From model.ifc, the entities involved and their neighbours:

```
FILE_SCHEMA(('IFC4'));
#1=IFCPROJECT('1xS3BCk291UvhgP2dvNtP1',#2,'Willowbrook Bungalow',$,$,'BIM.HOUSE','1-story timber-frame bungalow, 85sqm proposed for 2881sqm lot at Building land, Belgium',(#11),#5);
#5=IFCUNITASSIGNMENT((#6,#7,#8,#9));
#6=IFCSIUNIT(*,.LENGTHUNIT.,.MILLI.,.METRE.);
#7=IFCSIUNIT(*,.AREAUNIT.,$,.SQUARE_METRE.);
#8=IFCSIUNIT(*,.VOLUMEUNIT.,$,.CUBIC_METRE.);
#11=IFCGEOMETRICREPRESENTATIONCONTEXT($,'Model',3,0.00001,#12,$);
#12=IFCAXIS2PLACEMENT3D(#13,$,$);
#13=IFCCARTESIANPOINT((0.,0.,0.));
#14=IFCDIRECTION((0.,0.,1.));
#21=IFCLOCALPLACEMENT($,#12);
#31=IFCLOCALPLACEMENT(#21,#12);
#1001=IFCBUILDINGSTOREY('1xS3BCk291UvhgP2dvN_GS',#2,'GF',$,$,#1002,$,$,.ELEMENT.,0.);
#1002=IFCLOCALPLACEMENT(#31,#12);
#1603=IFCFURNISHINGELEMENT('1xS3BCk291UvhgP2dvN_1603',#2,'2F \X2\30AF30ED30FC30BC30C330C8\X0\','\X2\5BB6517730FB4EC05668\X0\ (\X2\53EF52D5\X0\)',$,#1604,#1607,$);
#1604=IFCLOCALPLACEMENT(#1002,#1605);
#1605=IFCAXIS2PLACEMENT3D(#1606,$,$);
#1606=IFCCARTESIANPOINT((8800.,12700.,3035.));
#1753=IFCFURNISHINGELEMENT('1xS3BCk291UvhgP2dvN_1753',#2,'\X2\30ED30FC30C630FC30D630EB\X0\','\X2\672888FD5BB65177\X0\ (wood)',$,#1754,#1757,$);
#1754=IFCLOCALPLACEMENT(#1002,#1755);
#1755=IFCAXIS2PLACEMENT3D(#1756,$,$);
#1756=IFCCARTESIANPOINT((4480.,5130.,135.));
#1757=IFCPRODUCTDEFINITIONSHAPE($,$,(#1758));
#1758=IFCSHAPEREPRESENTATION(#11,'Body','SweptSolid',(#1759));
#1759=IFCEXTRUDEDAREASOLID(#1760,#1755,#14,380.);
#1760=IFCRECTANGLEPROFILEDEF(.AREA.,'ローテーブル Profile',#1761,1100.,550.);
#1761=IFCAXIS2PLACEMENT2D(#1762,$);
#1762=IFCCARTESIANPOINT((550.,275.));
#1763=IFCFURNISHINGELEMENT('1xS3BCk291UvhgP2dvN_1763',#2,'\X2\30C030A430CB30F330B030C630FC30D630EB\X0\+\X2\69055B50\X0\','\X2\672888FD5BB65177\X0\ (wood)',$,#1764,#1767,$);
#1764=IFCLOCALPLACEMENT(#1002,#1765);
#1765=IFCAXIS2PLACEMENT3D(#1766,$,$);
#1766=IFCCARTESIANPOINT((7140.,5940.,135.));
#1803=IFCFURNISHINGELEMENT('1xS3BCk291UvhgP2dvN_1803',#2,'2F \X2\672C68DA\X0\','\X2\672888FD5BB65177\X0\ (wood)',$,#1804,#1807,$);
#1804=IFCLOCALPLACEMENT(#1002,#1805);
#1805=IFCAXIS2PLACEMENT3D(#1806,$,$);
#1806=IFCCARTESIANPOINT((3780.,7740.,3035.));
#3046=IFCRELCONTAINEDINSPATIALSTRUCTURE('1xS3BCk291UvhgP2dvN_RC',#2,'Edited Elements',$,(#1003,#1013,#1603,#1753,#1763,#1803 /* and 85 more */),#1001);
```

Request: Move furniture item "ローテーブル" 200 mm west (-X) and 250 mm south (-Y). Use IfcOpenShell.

```python
import ifcopenshell
import ifcopenshell.api.geometry
import ifcopenshell.util.placement
import ifcopenshell.util.unit

model = ifcopenshell.open("model.ifc")
unit_scale = ifcopenshell.util.unit.calculate_unit_scale(model)

item = model.by_id(1753)
matrix = ifcopenshell.util.placement.get_local_placement(item.ObjectPlacement)
matrix[0, 3] -= 0.2 / unit_scale
matrix[1, 3] -= 0.25 / unit_scale
ifcopenshell.api.geometry.edit_object_placement(model, product=item, matrix=matrix, is_si=False)

print(ifcopenshell.util.placement.get_local_placement(item.ObjectPlacement).round(3) + 0.0)

model.write("model_edited.ifc")
```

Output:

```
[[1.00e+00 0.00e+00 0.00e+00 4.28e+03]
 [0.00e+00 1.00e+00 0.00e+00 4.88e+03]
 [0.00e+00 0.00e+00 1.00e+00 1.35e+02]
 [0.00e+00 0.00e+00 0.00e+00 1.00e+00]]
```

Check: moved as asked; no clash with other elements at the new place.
